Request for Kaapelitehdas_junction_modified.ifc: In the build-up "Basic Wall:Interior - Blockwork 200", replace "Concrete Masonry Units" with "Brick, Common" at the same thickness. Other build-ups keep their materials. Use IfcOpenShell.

First a look at what the model holds.

```python
import ifcopenshell
import ifcopenshell.util.element

model = ifcopenshell.open("Kaapelitehdas_junction_modified.ifc")
print(model.schema)
for layer_set in model.by_type("IfcMaterialLayerSet"):
    if layer_set.LayerSetName == "Basic Wall:Interior - Blockwork 200":
        for layer in layer_set.MaterialLayers:
            print(layer.id(), layer.Material and layer.Material.Name, layer.LayerThickness, sep=" | ")
        print(len(ifcopenshell.util.element.get_elements_by_material(model, layer_set)), "elements and types use it")
print(sorted(m.Name for m in model.by_type("IfcMaterial") if m.Name)[:60])
```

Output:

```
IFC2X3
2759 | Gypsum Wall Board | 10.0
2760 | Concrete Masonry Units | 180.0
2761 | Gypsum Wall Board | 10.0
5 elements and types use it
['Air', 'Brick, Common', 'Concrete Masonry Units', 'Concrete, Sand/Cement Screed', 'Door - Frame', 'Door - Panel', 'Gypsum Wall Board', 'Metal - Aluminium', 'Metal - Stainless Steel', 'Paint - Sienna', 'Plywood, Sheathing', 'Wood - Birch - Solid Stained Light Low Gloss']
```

```python
import ifcopenshell
import ifcopenshell.api.material

model = ifcopenshell.open("Kaapelitehdas_junction_modified.ifc")

layer_set = next(s for s in model.by_type("IfcMaterialLayerSet") if s.LayerSetName == "Basic Wall:Interior - Blockwork 200")
layer = next(l for l in layer_set.MaterialLayers if l.Material and l.Material.Name == "Concrete Masonry Units")
material = next(m for m in model.by_type("IfcMaterial") if m.Name == "Brick, Common")

# Point this one layer at the other material; renaming the old one would change it everywhere.
ifcopenshell.api.material.edit_layer(model, layer=layer, attributes={}, material=material)

print([l.Material.Name if l.Material else None for l in layer_set.MaterialLayers])

model.write("Kaapelitehdas_junction_modified_rev.ifc")
```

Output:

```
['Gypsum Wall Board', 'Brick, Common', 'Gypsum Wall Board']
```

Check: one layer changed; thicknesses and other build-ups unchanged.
